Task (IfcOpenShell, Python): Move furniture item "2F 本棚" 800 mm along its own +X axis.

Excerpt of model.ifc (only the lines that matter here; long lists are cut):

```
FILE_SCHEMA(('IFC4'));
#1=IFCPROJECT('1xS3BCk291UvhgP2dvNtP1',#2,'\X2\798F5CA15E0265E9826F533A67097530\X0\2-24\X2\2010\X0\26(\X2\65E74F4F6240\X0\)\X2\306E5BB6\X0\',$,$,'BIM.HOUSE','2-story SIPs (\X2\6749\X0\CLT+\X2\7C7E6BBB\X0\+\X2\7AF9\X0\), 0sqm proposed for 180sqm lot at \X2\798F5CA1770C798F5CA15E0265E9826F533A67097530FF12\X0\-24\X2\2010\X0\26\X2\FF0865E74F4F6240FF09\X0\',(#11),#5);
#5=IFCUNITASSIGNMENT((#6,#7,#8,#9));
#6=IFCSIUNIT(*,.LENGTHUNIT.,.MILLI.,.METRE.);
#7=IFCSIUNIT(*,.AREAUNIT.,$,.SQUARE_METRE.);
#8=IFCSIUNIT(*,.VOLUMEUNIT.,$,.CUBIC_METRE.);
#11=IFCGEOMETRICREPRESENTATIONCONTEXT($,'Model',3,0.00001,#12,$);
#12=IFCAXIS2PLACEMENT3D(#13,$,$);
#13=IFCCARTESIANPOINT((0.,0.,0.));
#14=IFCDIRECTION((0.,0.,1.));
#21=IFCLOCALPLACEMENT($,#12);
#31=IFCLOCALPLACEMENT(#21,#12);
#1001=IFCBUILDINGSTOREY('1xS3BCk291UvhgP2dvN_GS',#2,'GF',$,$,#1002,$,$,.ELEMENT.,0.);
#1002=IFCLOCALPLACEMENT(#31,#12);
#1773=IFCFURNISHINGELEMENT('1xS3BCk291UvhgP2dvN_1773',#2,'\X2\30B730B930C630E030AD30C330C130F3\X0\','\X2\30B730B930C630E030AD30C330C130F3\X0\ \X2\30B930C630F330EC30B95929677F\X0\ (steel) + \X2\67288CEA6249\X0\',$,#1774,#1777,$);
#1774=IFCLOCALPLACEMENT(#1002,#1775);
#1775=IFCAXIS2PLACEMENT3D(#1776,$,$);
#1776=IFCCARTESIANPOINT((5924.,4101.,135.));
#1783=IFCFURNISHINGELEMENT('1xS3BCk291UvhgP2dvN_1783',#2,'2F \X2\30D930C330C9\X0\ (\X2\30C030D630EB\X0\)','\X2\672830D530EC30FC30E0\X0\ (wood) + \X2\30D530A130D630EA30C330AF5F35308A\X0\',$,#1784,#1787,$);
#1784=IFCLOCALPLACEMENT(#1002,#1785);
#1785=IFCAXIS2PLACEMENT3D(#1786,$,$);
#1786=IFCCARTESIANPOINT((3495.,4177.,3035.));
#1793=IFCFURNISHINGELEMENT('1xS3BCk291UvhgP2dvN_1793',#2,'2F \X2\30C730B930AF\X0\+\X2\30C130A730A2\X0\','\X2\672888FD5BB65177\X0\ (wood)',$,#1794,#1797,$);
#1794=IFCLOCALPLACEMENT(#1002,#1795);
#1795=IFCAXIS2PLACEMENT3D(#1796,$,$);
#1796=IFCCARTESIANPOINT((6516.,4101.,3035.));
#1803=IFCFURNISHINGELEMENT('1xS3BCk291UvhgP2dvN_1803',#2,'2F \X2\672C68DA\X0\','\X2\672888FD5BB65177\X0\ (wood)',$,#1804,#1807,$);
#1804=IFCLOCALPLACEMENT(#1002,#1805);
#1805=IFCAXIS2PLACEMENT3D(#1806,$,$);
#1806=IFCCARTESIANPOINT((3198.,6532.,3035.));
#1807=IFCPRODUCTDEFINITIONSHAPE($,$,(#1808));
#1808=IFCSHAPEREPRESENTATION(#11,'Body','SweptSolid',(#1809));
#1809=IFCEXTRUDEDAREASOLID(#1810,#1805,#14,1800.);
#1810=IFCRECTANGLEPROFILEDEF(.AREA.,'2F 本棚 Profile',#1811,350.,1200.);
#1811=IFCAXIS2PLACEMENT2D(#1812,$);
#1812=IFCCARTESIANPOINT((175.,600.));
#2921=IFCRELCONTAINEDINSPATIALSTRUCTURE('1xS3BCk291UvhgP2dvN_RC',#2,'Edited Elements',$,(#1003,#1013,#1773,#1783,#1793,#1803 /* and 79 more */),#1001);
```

```python
import ifcopenshell
import ifcopenshell.api.geometry
import ifcopenshell.util.placement
import ifcopenshell.util.unit

model = ifcopenshell.open("model.ifc")
unit_scale = ifcopenshell.util.unit.calculate_unit_scale(model)

item = model.by_guid("1xS3BCk291UvhgP2dvN_1803")
matrix = ifcopenshell.util.placement.get_local_placement(item.ObjectPlacement)
matrix[:3, 3] += matrix[:3, 0] * 0.8 / unit_scale
ifcopenshell.api.geometry.edit_object_placement(model, product=item, matrix=matrix, is_si=False)

print(ifcopenshell.util.placement.get_local_placement(item.ObjectPlacement).round(3) + 0.0)

model.write("model_updated.ifc")
```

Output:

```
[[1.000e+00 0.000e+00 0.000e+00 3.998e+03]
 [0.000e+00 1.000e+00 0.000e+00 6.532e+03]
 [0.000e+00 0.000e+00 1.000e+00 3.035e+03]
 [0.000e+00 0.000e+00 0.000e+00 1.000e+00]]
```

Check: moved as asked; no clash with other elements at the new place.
